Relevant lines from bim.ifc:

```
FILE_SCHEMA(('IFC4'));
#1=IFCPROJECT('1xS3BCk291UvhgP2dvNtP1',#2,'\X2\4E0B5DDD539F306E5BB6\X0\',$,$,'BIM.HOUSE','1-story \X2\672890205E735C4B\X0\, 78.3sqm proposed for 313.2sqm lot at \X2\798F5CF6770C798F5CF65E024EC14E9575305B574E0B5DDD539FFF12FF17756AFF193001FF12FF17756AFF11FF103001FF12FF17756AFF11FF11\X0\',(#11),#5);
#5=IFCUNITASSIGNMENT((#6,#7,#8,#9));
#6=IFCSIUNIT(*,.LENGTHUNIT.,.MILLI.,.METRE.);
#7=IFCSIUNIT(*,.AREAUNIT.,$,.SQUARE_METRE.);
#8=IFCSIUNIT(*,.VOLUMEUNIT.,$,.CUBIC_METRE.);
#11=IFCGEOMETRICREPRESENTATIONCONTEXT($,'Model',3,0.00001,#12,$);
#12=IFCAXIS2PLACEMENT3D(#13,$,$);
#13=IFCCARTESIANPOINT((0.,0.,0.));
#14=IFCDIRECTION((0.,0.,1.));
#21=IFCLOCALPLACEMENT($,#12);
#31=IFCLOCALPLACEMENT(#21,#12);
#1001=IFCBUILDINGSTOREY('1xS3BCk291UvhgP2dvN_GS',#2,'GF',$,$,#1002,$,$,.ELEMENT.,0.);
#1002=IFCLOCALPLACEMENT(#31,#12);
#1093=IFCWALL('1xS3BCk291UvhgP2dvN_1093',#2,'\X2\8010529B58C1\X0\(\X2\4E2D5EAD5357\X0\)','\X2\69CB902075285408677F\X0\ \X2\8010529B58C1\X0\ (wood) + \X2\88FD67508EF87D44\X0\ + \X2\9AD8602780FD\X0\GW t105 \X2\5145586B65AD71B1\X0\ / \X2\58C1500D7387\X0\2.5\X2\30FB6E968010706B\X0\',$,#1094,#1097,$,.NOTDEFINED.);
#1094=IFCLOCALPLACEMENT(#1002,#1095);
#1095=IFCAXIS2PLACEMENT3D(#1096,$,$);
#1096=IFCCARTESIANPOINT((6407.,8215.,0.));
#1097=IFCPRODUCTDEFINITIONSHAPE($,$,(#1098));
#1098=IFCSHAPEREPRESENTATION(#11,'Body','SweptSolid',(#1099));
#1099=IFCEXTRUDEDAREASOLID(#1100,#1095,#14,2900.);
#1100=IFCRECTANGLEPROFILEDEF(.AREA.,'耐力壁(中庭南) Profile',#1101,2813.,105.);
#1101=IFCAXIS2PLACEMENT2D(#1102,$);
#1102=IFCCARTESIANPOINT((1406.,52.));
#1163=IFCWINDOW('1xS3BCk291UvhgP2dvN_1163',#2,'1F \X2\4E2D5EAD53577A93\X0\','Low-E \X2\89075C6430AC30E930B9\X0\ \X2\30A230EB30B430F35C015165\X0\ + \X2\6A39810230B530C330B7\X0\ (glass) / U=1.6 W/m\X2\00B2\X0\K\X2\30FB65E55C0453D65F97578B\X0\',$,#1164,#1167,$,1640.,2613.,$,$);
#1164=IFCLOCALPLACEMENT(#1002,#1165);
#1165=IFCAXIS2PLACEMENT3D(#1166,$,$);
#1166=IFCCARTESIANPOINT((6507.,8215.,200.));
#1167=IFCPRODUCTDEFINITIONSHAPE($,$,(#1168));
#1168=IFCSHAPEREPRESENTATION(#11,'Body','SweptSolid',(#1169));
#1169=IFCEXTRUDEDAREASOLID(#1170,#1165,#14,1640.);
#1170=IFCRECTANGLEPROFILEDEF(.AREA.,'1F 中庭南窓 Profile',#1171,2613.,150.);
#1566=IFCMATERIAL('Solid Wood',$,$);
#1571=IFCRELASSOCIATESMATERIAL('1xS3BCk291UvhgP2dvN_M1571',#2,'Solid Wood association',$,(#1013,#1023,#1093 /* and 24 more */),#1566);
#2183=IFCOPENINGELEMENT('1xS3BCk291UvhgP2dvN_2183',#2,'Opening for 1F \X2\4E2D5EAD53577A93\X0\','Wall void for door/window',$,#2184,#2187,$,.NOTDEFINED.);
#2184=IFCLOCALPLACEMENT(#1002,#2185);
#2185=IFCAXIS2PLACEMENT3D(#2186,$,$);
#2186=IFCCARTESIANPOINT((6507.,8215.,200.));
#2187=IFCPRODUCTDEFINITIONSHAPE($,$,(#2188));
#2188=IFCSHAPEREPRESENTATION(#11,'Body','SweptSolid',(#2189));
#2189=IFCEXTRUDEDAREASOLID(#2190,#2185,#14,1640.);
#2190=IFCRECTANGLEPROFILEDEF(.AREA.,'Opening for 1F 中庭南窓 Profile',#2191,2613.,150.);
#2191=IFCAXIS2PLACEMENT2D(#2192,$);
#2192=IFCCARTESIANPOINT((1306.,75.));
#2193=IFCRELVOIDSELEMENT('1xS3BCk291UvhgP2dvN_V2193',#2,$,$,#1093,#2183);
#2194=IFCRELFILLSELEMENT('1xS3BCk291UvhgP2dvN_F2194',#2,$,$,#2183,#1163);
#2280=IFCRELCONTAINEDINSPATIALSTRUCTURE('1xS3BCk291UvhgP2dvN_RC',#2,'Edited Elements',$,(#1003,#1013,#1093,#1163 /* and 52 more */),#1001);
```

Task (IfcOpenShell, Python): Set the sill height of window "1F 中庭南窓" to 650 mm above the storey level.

```python
import numpy as np
import ifcopenshell
import ifcopenshell.api.geometry
import ifcopenshell.geom
import ifcopenshell.util.element
import ifcopenshell.util.placement
import ifcopenshell.util.shape
import ifcopenshell.util.unit

model = ifcopenshell.open("bim.ifc")
unit_scale = ifcopenshell.util.unit.calculate_unit_scale(model)

window = model.by_guid("1xS3BCk291UvhgP2dvN_1163")
opening = window.FillsVoids[0].RelatingOpeningElement
storey = ifcopenshell.util.element.get_container(window, ifc_class="IfcBuildingStorey")
level = ifcopenshell.util.placement.get_local_placement(storey.ObjectPlacement)[2, 3]

# The opening's origin need not be at the sill, so measure its lowest point.
shape = ifcopenshell.geom.create_shape(ifcopenshell.geom.settings(), opening)
bottom = ifcopenshell.util.shape.get_shape_bottom_elevation(shape, shape.geometry) / unit_scale
dz = level + 0.65 / unit_scale - bottom

shift = np.array([0.0, 0.0, dz])
# The window is not placed relative to its opening, so move both.
for product in (opening, window):
    matrix = ifcopenshell.util.placement.get_local_placement(product.ObjectPlacement)
    matrix[:3, 3] += shift
    ifcopenshell.api.geometry.edit_object_placement(model, product=product, matrix=matrix, is_si=False)

print(f"moved by {dz * unit_scale:+.3f} m")

model.write("bim-out.ifc")
```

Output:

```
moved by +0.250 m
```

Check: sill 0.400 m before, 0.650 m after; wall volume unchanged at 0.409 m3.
